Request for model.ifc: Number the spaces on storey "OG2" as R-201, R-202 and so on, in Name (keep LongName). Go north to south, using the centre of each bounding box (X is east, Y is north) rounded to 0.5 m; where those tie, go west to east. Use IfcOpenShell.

First a look at what the model holds.

```python
import ifcopenshell
import ifcopenshell.util.element
import ifcopenshell.util.placement

model = ifcopenshell.open("model.ifc")
print(model.schema)
storey = next(s for s in model.by_type("IfcBuildingStorey") if s.Name == "OG2")
spaces = [e for e in ifcopenshell.util.element.get_decomposition(storey) if e.is_a("IfcSpace")]
for e in sorted(spaces, key=lambda e: e.id()):
    origin = ifcopenshell.util.placement.get_local_placement(e.ObjectPlacement)[:3, 3]
    print(e.id(), e.Name, e.LongName, origin.round(2) + 0.0, sep=" | ")
```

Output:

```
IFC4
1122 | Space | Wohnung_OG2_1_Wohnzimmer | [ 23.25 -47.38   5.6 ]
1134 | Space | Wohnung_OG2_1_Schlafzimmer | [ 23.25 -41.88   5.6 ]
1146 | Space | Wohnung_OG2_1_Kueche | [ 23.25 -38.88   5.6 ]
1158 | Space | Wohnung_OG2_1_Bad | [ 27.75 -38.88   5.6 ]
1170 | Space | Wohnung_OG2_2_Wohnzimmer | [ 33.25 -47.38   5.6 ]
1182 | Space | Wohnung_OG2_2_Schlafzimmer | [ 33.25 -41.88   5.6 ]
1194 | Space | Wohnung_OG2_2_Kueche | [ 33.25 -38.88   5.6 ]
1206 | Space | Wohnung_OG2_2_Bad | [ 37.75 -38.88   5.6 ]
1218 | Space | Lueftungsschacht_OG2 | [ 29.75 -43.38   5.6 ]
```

```python
import ifcopenshell
import ifcopenshell.geom
import ifcopenshell.util.element
import ifcopenshell.util.shape

model = ifcopenshell.open("model.ifc")
settings = ifcopenshell.geom.settings()
settings.set("use-world-coords", True)


def centre(element):
    shape = ifcopenshell.geom.create_shape(settings, element)
    return ifcopenshell.util.shape.get_bbox_centroid(shape.geometry)


storey = next(s for s in model.by_type("IfcBuildingStorey") if s.Name == "OG2")
spaces = [e for e in ifcopenshell.util.element.get_decomposition(storey) if e.is_a("IfcSpace")]

# Insertion points can sit at a corner or the storey origin, so sort by the geometry (in metres).
centres = {e: centre(e) for e in spaces}
spaces.sort(key=lambda e: (-round(centres[e][1] / 0.5), centres[e][0]))

for i, e in enumerate(spaces, start=1):
    number = f"R-2{i:02d}"
    e.Name = number
    print(e.id(), number)

model.write("model-out.ifc")
```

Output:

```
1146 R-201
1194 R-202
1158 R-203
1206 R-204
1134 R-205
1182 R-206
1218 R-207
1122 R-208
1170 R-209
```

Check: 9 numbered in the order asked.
